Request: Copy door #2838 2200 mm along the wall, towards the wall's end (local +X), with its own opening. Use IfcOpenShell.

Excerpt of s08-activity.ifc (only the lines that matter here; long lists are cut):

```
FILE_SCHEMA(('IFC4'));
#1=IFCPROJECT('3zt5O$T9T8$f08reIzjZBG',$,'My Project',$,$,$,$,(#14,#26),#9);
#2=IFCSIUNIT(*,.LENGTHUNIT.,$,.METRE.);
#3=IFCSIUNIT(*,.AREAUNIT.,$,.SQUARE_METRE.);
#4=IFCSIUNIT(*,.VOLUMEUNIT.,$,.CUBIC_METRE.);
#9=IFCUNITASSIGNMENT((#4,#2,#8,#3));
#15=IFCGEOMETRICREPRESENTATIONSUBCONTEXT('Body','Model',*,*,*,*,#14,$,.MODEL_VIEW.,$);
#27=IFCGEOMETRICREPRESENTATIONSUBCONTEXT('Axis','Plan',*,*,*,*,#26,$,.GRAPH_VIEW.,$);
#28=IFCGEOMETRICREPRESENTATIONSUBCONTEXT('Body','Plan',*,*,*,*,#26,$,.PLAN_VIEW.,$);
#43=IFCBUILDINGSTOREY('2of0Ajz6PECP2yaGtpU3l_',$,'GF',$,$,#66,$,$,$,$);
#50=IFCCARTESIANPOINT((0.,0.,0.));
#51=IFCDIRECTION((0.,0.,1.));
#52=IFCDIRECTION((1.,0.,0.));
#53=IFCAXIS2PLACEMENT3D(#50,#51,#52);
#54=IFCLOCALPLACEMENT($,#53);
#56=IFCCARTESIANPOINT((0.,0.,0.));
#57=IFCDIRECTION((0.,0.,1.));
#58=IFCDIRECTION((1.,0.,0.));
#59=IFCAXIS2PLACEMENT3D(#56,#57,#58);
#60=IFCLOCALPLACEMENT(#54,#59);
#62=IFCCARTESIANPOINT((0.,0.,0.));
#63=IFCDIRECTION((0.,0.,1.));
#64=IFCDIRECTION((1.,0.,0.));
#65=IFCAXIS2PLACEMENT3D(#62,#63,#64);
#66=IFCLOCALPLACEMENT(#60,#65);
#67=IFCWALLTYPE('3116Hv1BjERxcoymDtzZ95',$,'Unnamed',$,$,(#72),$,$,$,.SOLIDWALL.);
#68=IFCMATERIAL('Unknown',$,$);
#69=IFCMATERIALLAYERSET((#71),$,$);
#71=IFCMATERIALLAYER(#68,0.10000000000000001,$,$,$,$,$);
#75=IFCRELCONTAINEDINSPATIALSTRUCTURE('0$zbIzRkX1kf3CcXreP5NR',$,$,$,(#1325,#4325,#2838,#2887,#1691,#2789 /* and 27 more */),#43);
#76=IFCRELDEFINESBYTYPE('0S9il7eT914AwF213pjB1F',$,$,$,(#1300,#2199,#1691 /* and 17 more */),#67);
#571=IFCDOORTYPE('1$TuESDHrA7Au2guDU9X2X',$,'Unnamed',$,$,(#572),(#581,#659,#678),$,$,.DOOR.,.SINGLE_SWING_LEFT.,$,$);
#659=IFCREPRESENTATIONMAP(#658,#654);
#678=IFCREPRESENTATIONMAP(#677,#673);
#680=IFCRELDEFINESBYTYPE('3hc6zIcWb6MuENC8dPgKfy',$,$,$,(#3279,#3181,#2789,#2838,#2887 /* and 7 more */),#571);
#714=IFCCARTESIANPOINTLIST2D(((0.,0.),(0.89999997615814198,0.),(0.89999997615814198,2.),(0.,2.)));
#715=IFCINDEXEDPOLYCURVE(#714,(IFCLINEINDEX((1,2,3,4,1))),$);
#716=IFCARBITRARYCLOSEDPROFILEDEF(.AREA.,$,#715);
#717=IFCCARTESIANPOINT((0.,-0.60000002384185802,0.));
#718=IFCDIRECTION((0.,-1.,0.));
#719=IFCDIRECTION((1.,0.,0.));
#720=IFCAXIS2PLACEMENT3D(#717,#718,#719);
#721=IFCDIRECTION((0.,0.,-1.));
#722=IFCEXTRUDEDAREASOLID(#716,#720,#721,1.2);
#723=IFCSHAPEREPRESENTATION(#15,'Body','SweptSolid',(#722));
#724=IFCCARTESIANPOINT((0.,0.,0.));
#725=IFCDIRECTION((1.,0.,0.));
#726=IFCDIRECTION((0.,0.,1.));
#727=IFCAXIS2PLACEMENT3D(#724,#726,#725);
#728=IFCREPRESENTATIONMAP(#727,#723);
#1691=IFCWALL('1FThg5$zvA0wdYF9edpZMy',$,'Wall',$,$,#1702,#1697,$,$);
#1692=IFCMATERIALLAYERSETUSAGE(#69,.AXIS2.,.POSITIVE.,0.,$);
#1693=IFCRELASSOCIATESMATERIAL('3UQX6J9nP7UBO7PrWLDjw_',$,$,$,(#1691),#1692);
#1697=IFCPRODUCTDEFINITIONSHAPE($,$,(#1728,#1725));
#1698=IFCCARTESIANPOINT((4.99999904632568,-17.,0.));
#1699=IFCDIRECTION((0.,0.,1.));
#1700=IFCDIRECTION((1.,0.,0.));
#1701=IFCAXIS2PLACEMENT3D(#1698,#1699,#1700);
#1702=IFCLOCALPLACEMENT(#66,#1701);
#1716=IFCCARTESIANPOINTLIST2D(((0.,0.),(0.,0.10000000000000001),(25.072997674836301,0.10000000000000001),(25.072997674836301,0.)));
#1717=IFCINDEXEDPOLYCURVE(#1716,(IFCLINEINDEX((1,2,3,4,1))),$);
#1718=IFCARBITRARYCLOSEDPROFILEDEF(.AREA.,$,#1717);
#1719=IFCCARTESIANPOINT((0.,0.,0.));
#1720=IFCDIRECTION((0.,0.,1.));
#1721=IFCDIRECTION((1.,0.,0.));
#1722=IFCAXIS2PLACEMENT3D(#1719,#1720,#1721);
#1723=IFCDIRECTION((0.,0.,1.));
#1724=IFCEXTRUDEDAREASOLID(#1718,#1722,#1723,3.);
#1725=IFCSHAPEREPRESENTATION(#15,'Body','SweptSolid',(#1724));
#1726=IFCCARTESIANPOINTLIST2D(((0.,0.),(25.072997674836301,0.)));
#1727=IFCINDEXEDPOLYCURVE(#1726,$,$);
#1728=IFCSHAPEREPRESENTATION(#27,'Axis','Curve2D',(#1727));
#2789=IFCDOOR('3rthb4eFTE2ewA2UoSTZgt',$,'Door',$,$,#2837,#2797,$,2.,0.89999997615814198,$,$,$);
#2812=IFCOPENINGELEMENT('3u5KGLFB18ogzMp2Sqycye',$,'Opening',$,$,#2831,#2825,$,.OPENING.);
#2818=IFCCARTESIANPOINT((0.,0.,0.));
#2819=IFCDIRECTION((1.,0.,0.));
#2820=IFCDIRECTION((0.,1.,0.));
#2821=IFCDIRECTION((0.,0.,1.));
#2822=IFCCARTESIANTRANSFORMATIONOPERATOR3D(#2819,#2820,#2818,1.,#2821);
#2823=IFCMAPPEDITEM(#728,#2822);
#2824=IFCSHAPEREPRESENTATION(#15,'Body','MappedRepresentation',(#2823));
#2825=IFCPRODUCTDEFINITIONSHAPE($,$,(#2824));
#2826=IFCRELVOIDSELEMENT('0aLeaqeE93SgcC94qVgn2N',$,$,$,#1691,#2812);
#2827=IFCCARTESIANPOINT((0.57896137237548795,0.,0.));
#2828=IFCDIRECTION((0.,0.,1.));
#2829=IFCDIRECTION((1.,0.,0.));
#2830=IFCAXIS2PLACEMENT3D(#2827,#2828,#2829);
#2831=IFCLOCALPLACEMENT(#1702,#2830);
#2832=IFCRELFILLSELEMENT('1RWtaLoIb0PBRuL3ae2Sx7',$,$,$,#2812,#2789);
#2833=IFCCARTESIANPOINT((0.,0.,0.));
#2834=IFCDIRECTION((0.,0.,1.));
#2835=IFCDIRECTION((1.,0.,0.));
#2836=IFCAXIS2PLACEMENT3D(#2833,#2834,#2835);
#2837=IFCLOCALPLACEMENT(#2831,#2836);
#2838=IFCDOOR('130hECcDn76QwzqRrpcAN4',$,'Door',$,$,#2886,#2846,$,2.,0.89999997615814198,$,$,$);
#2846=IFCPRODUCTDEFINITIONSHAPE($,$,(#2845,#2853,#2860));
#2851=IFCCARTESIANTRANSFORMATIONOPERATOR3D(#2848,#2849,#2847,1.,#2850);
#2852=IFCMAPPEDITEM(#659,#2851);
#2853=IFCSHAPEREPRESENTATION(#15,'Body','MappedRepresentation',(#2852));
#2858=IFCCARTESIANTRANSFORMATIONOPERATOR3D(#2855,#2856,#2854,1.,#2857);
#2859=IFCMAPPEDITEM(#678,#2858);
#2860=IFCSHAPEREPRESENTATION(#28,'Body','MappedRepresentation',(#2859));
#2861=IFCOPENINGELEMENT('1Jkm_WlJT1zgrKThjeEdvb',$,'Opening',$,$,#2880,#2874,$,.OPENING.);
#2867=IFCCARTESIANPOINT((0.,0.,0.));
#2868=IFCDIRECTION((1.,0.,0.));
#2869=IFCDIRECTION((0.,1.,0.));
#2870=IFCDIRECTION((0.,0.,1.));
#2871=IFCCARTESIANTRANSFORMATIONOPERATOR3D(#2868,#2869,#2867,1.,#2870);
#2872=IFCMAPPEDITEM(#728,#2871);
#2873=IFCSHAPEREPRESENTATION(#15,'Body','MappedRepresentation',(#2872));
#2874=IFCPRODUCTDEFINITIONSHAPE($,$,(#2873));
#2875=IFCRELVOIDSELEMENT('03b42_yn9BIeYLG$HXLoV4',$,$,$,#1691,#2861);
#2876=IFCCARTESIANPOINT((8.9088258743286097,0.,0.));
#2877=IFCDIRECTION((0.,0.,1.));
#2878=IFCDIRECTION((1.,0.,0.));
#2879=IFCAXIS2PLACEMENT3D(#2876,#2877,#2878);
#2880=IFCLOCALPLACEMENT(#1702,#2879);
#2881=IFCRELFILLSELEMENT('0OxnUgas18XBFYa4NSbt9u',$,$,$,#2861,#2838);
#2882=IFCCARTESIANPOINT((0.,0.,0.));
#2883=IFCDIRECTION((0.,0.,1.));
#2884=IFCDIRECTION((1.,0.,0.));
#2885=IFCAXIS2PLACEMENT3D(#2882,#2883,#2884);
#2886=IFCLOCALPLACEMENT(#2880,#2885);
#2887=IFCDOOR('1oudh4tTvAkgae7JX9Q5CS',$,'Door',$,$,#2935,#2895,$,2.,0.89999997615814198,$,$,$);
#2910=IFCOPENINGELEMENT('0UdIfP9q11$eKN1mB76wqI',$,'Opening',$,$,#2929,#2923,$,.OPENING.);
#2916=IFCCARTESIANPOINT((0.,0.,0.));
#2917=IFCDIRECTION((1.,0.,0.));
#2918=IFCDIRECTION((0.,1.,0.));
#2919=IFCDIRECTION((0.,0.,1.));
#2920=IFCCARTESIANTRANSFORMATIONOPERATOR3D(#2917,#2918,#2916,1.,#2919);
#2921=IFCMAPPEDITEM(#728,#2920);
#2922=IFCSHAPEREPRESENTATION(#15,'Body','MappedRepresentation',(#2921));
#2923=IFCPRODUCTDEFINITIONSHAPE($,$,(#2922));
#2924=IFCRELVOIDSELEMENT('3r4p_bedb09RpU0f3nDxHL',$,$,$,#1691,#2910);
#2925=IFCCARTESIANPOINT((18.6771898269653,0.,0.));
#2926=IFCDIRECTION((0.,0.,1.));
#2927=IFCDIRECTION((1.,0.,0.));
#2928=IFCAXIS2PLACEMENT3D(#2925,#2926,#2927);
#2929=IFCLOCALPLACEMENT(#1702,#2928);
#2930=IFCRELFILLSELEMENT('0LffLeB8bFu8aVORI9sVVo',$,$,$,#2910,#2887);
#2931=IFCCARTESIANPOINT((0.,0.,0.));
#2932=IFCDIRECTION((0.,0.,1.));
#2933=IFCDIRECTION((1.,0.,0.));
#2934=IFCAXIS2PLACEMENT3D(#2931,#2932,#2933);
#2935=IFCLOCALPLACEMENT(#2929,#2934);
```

```python
import ifcopenshell
import ifcopenshell.api.feature
import ifcopenshell.api.geometry
import ifcopenshell.api.root
import ifcopenshell.geom
import ifcopenshell.util.element
import ifcopenshell.util.placement
import ifcopenshell.util.shape

model = ifcopenshell.open("s08-activity.ifc")
settings = ifcopenshell.geom.settings()


def volume(element):
    """Net volume in cubic metres, openings subtracted."""
    shape = ifcopenshell.geom.create_shape(settings, element)
    return ifcopenshell.util.shape.get_volume(shape.geometry)


door = model.by_id(2838)
opening = door.FillsVoids[0].RelatingOpeningElement
wall = opening.VoidsElements[0].RelatingBuildingElement
before = volume(wall)
shift = ifcopenshell.util.placement.get_local_placement(wall.ObjectPlacement)[:3, 0] * 2.2

# copy_class copies the void relationship, type, container and properties, but no geometry.
new_opening = ifcopenshell.api.root.copy_class(model, product=opening)
new_opening.Representation = ifcopenshell.util.element.copy_deep(
    model, opening.Representation, exclude=["IfcGeometricRepresentationContext", "IfcRepresentationMap"]
)
new_door = ifcopenshell.api.root.copy_class(model, product=door)
new_door.Representation = ifcopenshell.util.element.copy_deep(
    model, door.Representation, exclude=["IfcGeometricRepresentationContext", "IfcRepresentationMap"]
)
ifcopenshell.api.feature.add_filling(model, opening=new_opening, element=new_door)

for old, new in ((opening, new_opening), (door, new_door)):
    matrix = ifcopenshell.util.placement.get_local_placement(old.ObjectPlacement)
    matrix[:3, 3] += shift
    ifcopenshell.api.geometry.edit_object_placement(model, product=new, matrix=matrix, is_si=False)

after = volume(wall)

print(f"wall volume {before:.3f} -> {after:.3f} m3")

model.write("s08-activity_v2.ifc")
```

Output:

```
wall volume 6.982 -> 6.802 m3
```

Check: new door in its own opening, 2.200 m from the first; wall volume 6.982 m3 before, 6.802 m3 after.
